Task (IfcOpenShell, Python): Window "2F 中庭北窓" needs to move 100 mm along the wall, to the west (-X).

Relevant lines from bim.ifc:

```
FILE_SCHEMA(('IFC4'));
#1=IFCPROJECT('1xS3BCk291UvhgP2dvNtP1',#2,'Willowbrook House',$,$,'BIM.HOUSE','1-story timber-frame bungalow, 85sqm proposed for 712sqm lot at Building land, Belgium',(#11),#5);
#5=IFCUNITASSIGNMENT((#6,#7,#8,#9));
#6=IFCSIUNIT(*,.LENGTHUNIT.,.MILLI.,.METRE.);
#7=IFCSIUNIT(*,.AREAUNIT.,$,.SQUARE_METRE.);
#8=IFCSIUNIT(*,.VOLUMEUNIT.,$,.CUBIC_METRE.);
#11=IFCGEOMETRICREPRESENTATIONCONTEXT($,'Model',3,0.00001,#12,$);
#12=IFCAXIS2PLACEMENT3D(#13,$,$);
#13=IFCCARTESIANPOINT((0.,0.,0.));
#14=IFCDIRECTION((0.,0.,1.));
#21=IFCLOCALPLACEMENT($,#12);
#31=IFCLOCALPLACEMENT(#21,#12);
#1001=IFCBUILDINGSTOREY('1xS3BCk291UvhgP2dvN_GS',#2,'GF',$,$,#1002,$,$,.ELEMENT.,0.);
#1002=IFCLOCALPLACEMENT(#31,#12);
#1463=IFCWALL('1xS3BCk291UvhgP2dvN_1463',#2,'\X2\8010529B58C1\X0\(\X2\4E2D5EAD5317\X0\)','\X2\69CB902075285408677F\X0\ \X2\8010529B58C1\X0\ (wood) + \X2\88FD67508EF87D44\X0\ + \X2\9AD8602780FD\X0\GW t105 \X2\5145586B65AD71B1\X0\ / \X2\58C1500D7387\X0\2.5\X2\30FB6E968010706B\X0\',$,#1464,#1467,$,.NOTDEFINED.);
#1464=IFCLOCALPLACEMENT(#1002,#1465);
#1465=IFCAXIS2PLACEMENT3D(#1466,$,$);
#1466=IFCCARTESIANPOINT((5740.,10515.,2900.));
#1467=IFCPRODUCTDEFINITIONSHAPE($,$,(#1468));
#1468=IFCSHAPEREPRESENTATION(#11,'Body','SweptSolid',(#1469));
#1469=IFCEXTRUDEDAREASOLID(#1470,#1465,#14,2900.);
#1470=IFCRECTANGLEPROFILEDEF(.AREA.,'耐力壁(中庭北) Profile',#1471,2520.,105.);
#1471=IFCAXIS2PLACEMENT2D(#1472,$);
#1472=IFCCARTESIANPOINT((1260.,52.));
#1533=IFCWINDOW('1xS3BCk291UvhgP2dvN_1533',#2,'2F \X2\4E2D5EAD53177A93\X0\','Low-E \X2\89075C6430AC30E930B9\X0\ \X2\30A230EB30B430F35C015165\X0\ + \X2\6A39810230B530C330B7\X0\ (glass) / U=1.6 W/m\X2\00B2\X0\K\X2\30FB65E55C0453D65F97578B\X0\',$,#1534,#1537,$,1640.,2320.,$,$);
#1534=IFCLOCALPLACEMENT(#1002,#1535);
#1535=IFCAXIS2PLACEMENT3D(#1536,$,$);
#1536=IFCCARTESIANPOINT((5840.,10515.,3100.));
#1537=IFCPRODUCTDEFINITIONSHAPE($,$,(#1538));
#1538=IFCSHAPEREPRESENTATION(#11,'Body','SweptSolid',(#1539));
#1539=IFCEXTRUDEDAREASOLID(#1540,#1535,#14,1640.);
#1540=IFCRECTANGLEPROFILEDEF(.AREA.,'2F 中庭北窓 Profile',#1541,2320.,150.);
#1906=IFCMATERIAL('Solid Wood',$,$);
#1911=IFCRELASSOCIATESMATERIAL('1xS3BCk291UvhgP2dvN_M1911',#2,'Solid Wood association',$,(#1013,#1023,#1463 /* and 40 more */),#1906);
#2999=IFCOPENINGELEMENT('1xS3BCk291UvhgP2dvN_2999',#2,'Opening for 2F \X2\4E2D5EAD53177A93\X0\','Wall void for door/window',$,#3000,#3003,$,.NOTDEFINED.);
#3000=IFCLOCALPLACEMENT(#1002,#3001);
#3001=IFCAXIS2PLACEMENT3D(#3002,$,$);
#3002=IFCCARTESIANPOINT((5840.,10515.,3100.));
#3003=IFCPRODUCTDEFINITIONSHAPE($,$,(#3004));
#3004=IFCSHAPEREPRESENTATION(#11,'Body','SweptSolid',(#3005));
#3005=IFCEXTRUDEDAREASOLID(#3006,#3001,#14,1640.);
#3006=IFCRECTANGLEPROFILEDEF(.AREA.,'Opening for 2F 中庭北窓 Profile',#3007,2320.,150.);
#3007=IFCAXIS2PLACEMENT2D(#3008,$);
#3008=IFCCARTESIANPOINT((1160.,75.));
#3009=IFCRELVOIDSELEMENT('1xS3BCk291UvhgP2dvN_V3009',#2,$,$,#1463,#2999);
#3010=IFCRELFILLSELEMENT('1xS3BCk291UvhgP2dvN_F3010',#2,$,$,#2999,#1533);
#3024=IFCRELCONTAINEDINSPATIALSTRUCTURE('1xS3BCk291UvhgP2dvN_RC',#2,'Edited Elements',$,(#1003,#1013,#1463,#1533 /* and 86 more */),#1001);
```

```python
import ifcopenshell
import ifcopenshell.api.geometry
import ifcopenshell.util.placement
import ifcopenshell.util.unit

model = ifcopenshell.open("bim.ifc")
unit_scale = ifcopenshell.util.unit.calculate_unit_scale(model)

window = model.by_id(1533)
opening = window.FillsVoids[0].RelatingOpeningElement
wall = opening.VoidsElements[0].RelatingBuildingElement

wall_matrix = ifcopenshell.util.placement.get_local_placement(wall.ObjectPlacement)
shift = wall_matrix[:3, 0] * -0.1 / unit_scale
before = ifcopenshell.util.placement.get_local_placement(window.ObjectPlacement)[:3, 3].copy()

# The window is not placed relative to its opening, so move both.
for product in (opening, window):
    matrix = ifcopenshell.util.placement.get_local_placement(product.ObjectPlacement)
    matrix[:3, 3] += shift
    ifcopenshell.api.geometry.edit_object_placement(model, product=product, matrix=matrix, is_si=False)

after = ifcopenshell.util.placement.get_local_placement(window.ObjectPlacement)[:3, 3]
print("window moved by", (after - before).round(3) + 0.0)

model.write("bim_v2.ifc")
```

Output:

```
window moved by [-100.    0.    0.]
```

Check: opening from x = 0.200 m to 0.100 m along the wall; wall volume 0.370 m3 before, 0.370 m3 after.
